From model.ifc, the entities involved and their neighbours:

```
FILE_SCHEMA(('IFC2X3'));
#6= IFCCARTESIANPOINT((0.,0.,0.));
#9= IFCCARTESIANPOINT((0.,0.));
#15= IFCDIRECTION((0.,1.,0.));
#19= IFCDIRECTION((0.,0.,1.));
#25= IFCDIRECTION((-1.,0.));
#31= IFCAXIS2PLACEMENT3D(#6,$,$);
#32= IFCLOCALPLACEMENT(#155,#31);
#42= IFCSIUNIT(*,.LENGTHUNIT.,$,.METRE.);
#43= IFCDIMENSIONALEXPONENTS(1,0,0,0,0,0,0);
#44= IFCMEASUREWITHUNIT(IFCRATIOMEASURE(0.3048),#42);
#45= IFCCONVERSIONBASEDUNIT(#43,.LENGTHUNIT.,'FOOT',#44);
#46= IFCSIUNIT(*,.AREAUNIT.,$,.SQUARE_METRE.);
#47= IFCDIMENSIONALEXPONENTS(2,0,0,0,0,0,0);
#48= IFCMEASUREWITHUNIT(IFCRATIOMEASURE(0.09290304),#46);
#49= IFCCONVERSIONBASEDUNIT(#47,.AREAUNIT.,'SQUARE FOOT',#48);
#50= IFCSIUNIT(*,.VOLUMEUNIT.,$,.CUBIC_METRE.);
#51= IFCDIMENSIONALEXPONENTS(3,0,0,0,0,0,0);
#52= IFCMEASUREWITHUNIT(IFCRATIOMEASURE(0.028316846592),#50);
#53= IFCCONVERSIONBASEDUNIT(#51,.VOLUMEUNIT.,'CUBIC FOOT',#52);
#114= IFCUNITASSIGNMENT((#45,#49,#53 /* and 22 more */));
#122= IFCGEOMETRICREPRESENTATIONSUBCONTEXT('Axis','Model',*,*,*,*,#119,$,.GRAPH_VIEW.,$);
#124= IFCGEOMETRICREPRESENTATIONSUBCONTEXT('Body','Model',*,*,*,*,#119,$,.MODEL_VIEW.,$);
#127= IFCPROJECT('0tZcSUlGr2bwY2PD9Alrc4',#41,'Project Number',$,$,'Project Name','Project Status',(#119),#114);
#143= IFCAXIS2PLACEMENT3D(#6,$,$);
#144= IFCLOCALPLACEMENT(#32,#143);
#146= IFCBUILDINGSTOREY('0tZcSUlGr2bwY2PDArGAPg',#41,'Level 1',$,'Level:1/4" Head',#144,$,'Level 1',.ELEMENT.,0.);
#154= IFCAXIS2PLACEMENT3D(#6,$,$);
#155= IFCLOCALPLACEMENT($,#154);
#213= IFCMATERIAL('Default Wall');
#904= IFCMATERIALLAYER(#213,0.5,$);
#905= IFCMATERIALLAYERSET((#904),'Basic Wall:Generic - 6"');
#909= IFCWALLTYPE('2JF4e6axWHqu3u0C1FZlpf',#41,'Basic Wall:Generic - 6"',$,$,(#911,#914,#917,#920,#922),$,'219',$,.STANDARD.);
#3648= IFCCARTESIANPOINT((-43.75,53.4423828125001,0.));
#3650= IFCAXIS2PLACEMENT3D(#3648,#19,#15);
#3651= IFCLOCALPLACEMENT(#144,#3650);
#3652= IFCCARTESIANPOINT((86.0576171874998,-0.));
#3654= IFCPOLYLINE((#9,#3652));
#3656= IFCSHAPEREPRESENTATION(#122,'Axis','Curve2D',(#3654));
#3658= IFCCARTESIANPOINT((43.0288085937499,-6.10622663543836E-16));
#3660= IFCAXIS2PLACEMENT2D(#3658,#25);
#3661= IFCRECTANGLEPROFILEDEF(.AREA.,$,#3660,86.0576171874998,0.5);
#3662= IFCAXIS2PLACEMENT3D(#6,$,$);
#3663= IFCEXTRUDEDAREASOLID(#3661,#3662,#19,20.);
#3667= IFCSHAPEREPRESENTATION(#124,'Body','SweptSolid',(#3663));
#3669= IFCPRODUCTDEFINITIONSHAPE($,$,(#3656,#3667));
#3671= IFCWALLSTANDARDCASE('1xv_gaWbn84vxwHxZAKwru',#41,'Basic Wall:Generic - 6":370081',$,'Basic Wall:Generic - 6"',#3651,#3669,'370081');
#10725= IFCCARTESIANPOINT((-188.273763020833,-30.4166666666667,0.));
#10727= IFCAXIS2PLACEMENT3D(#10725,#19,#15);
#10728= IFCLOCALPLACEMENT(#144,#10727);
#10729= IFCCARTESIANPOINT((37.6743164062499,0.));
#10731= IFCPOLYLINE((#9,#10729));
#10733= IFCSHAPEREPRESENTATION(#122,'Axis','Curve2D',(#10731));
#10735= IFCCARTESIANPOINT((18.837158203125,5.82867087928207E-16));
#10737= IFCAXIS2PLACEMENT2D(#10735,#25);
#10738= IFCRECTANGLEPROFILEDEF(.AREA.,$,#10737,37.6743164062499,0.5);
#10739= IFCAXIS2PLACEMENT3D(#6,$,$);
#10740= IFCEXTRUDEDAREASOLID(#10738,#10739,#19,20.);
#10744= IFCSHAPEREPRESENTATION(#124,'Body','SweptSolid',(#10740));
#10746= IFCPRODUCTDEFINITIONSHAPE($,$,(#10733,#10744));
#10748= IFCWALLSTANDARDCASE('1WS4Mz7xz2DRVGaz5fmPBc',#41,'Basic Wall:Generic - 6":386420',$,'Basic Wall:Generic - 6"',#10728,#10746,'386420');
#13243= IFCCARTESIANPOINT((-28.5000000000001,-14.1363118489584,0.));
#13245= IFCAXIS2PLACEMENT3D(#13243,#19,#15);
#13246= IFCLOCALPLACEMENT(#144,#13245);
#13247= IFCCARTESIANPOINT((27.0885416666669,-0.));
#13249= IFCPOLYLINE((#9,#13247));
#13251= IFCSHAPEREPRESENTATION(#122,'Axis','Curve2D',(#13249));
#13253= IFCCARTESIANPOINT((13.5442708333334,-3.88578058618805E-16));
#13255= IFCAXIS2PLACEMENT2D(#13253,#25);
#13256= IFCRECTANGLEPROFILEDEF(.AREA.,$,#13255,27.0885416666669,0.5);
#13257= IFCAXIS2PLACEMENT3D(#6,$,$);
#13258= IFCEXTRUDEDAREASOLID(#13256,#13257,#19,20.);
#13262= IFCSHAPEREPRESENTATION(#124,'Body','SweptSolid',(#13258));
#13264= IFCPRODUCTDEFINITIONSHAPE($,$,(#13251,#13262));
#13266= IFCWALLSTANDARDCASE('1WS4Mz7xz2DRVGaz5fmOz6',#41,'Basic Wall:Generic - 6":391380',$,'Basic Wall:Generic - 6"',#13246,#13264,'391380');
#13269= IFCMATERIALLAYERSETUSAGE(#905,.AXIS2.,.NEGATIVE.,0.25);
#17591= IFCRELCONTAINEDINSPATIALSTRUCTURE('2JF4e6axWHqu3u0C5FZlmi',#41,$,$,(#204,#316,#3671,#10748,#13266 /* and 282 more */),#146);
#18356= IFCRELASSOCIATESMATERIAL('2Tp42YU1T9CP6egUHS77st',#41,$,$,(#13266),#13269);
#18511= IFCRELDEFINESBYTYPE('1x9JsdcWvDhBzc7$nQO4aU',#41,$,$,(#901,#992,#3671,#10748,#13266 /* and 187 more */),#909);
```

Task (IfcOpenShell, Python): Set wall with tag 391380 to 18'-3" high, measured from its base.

```python
import ifcopenshell
import ifcopenshell.geom
import ifcopenshell.util.representation
import ifcopenshell.util.shape
import ifcopenshell.util.unit

model = ifcopenshell.open("model.ifc")
unit_scale = ifcopenshell.util.unit.calculate_unit_scale(model)
settings = ifcopenshell.geom.settings()


def volume(element):
    """Net volume in cubic metres, openings subtracted."""
    shape = ifcopenshell.geom.create_shape(settings, element)
    return ifcopenshell.util.shape.get_volume(shape.geometry)


wall = model.by_guid("1WS4Mz7xz2DRVGaz5fmOz6")
before = volume(wall)

body = ifcopenshell.util.representation.get_representation(wall, "Model", "Body")
solid = body.Items[0]
old_height = solid.Depth
solid.Depth = 219 * 0.0254 / unit_scale
after = volume(wall)

print(f"height {old_height:g} -> {solid.Depth:g}, volume {before:.3f} -> {after:.3f} m3")

model.write("model-out.ifc")
```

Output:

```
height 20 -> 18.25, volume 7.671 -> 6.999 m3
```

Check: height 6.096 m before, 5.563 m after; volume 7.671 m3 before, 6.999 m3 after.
